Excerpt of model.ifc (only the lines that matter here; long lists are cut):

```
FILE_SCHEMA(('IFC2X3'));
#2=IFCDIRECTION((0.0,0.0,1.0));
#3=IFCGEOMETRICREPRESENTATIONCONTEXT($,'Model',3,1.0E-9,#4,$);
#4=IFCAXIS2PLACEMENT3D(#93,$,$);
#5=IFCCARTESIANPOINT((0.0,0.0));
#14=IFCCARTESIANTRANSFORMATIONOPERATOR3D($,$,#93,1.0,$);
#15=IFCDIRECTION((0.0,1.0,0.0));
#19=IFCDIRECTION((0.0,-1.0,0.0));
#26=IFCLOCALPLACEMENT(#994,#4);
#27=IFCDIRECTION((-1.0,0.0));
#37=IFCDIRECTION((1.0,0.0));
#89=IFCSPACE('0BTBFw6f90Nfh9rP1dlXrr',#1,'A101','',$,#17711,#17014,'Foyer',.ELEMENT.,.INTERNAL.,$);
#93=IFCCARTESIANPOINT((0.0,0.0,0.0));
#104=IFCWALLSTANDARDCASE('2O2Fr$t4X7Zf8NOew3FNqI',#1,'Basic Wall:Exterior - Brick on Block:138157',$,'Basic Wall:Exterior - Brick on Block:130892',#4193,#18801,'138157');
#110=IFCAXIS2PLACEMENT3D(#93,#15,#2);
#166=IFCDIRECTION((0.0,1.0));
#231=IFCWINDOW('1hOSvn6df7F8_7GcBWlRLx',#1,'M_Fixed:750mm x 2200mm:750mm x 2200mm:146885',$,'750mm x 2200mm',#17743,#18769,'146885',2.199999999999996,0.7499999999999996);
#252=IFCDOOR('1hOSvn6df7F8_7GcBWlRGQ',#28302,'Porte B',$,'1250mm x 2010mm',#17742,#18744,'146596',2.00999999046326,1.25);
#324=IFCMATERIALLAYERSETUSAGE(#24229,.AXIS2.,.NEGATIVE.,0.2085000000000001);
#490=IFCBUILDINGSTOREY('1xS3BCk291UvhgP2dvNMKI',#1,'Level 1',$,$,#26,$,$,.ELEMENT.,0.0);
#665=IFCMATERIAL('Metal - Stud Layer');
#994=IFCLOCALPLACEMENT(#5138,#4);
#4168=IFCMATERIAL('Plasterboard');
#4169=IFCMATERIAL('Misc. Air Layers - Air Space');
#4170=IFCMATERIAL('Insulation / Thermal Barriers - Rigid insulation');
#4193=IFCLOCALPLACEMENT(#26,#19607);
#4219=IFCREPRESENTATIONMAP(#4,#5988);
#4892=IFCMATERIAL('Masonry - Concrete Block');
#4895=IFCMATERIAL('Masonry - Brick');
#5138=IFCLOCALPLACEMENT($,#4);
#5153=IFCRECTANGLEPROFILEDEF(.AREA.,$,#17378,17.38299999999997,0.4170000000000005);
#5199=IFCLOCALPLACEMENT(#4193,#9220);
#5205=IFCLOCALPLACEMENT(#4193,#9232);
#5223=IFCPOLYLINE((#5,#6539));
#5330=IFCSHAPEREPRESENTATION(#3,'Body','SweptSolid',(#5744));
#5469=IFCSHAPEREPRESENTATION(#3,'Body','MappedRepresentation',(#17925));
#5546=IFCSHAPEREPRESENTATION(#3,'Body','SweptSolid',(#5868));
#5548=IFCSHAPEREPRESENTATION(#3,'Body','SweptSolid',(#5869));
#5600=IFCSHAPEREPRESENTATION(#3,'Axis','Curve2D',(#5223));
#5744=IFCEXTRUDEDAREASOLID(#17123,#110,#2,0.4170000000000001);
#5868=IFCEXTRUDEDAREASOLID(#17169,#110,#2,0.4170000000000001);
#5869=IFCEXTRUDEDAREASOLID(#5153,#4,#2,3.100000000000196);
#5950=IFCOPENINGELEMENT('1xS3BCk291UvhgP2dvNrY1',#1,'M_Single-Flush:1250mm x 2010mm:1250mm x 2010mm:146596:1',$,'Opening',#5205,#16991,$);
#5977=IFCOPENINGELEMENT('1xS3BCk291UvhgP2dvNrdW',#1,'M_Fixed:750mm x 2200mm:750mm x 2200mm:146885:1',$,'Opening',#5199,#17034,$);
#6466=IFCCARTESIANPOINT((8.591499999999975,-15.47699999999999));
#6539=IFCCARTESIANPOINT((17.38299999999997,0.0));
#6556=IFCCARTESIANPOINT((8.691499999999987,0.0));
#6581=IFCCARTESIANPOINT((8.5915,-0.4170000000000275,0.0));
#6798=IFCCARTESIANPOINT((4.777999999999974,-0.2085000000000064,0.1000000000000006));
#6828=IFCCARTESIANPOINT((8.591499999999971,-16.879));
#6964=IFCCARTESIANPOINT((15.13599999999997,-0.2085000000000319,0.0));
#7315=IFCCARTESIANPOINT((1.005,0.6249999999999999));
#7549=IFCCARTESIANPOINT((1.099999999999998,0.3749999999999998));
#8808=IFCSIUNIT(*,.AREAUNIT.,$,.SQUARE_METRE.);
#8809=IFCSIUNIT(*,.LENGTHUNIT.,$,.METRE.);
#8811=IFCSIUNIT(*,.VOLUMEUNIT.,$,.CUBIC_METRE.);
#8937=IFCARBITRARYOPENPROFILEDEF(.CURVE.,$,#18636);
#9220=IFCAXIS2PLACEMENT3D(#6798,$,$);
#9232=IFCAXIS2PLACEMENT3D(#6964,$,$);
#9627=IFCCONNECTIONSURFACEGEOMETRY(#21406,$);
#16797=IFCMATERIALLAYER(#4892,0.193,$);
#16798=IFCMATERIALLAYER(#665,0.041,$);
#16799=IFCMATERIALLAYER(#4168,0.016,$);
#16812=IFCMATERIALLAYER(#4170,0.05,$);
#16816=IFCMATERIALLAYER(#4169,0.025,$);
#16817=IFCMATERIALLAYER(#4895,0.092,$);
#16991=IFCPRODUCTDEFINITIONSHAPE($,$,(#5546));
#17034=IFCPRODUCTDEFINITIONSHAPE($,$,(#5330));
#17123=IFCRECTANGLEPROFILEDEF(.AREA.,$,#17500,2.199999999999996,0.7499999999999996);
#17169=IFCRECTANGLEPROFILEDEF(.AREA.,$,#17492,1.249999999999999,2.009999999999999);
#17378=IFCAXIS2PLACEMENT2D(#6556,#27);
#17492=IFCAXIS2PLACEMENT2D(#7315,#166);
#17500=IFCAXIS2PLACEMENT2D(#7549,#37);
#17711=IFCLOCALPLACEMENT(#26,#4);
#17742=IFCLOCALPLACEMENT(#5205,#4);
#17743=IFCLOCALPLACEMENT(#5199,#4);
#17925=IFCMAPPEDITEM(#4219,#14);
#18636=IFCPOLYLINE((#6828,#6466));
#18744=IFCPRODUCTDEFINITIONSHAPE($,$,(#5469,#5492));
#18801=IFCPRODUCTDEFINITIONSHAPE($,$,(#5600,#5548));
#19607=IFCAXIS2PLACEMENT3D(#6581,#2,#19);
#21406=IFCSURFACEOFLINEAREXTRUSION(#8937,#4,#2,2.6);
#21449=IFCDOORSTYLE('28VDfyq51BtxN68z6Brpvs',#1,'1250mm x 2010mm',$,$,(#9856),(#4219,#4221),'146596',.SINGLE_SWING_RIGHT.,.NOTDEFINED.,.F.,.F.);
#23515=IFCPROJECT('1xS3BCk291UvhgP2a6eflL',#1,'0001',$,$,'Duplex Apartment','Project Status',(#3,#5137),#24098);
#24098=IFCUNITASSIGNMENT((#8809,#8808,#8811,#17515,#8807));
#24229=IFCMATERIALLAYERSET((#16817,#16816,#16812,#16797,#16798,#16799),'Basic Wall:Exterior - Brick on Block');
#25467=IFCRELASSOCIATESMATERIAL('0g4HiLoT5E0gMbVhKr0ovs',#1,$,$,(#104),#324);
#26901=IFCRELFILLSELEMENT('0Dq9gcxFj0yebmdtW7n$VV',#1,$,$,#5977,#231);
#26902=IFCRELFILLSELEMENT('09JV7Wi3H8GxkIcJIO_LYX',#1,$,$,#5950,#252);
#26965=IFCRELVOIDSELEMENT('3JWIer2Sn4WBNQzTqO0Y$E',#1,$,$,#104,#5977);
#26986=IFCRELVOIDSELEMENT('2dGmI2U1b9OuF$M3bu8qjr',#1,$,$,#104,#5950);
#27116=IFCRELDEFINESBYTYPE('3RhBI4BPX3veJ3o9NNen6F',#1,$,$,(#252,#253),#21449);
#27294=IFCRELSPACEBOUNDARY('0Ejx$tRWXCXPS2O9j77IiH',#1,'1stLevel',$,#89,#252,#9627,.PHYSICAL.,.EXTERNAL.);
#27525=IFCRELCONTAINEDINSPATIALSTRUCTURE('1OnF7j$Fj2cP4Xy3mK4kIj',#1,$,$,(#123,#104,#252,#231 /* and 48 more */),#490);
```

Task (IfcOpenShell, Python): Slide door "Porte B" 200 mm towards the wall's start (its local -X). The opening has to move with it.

```python
import numpy as np
import ifcopenshell
import ifcopenshell.api.geometry
import ifcopenshell.util.placement

model = ifcopenshell.open("model.ifc")

door = model.by_guid("1hOSvn6df7F8_7GcBWlRGQ")
opening = door.FillsVoids[0].RelatingOpeningElement
wall = opening.VoidsElements[0].RelatingBuildingElement

wall_matrix = ifcopenshell.util.placement.get_local_placement(wall.ObjectPlacement)
shift = wall_matrix[:3, 0] * -0.2
before = ifcopenshell.util.placement.get_local_placement(door.ObjectPlacement)[:3, 3].copy()

# The door is placed relative to its opening, so it follows when the opening moves.
matrix = ifcopenshell.util.placement.get_local_placement(opening.ObjectPlacement)
matrix[:3, 3] += shift
ifcopenshell.api.geometry.edit_object_placement(
    model, product=opening, matrix=matrix, is_si=False, should_transform_children=True
)

# Space boundary surfaces are stored in each space's coordinates; move them too.
for rel in door.ProvidesBoundaries:
    if not rel.ConnectionGeometry:
        continue
    surface = rel.ConnectionGeometry.SurfaceOnRelatingElement
    space_matrix = ifcopenshell.util.placement.get_local_placement(rel.RelatingSpace.ObjectPlacement)
    point = np.array(surface.Position.Location.Coordinates) + space_matrix[:3, :3].T @ shift
    surface.Position = model.createIfcAxis2Placement3D(
        model.createIfcCartesianPoint(point.tolist()), surface.Position.Axis, surface.Position.RefDirection
    )

after = ifcopenshell.util.placement.get_local_placement(door.ObjectPlacement)[:3, 3]
print("door moved by", (after - before).round(3) + 0.0)

model.write("model-out.ifc")
```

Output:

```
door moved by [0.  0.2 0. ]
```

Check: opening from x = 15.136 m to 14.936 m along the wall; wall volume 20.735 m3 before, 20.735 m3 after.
